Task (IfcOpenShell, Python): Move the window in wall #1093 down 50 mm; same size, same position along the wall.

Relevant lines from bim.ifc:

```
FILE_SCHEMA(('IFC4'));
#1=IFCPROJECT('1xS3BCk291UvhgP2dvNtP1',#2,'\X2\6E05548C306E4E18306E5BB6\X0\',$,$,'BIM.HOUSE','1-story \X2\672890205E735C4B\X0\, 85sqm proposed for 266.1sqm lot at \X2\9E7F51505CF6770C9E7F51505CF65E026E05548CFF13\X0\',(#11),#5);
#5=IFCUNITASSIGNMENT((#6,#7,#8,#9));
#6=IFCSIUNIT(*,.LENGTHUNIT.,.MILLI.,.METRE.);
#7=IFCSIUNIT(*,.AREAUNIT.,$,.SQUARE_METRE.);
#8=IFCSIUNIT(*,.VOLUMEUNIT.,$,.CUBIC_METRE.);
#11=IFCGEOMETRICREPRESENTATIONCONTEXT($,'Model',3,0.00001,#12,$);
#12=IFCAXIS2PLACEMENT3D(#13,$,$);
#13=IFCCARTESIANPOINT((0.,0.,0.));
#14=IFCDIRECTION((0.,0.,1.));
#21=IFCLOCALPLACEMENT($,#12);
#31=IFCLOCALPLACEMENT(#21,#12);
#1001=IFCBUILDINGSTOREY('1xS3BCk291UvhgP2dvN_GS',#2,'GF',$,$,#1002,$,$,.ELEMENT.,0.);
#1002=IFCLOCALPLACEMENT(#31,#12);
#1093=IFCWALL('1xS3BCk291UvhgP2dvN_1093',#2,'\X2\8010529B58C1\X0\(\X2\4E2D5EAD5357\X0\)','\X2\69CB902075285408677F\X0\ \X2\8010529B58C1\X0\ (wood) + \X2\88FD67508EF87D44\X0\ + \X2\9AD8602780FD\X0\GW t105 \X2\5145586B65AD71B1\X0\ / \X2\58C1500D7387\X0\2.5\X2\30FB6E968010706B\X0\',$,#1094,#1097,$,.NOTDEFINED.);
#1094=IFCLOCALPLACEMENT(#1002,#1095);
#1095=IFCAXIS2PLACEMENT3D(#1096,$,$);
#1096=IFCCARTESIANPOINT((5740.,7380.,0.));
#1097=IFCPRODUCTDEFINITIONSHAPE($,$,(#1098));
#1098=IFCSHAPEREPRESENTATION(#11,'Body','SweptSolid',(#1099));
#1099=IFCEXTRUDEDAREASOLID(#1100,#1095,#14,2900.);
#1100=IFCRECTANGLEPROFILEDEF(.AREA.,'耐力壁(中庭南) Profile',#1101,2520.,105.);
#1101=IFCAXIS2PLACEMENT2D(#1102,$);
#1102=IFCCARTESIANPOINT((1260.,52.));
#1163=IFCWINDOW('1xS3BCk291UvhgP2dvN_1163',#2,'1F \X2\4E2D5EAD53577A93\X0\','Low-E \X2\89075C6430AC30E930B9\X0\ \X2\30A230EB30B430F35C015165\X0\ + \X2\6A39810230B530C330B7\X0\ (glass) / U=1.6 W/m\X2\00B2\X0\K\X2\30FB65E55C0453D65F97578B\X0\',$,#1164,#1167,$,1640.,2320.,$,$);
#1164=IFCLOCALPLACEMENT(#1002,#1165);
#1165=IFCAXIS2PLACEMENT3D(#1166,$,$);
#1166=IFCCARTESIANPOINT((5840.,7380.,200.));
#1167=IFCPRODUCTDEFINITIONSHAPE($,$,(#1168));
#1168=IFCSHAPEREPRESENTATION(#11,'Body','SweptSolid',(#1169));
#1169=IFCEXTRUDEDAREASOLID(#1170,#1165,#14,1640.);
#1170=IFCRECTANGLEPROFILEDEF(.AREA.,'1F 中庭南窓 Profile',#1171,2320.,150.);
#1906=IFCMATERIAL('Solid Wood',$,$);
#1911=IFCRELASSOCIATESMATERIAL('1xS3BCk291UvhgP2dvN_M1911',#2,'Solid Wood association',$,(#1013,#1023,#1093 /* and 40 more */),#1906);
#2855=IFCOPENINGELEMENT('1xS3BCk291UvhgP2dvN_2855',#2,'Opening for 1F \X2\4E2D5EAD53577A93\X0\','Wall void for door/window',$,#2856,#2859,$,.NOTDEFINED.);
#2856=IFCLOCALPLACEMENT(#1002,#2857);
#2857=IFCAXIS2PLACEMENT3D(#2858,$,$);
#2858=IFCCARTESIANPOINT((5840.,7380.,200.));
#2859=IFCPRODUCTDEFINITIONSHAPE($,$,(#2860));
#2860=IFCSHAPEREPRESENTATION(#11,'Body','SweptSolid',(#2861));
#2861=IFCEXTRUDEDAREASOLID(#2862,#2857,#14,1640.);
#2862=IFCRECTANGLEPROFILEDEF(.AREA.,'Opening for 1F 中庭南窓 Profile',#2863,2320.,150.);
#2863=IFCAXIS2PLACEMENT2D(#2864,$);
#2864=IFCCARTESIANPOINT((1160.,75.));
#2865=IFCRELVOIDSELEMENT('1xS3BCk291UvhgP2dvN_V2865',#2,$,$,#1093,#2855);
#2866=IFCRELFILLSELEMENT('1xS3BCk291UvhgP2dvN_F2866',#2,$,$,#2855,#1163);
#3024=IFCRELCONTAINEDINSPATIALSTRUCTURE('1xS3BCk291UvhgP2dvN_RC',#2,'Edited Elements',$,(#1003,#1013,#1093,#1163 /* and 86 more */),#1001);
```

```python
import numpy as np
import ifcopenshell
import ifcopenshell.api.geometry
import ifcopenshell.util.placement
import ifcopenshell.util.unit

model = ifcopenshell.open("bim.ifc")
unit_scale = ifcopenshell.util.unit.calculate_unit_scale(model)

window = model.by_id(1163)
opening = window.FillsVoids[0].RelatingOpeningElement
dz = -50.0

shift = np.array([0.0, 0.0, dz])
# The window is not placed relative to its opening, so move both.
for product in (opening, window):
    matrix = ifcopenshell.util.placement.get_local_placement(product.ObjectPlacement)
    matrix[:3, 3] += shift
    ifcopenshell.api.geometry.edit_object_placement(model, product=product, matrix=matrix, is_si=False)

print(f"moved by {dz * unit_scale:+.3f} m")

model.write("bim_updated.ifc")
```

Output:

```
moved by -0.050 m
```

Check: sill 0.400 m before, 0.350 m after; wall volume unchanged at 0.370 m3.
